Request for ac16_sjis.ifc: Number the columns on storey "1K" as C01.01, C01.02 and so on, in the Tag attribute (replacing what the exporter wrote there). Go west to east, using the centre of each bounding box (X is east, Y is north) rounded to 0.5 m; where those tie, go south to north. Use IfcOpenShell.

First a look at what the model holds.

```python
import ifcopenshell
import ifcopenshell.util.element
import ifcopenshell.util.placement

model = ifcopenshell.open("ac16_sjis.ifc")
print(model.schema)
storey = next(s for s in model.by_type("IfcBuildingStorey") if s.Name == '1\x8aK')
columns = [e for e in ifcopenshell.util.element.get_decomposition(storey) if e.is_a("IfcColumn")]
for e in sorted(columns, key=lambda e: e.id()):
    origin = ifcopenshell.util.placement.get_local_placement(e.ObjectPlacement)[:3, 3]
    print(e.id(), e.Tag, e.Name, origin.round(2) + 0.0, sep=" | ")
```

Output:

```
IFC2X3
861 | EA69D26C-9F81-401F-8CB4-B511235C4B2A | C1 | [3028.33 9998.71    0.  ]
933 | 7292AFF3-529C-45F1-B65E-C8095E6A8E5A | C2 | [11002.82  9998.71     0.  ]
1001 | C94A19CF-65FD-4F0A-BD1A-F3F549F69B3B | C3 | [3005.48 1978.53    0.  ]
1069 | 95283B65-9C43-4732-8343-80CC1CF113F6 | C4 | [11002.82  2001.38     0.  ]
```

```python
import ifcopenshell
import ifcopenshell.geom
import ifcopenshell.util.element
import ifcopenshell.util.shape

model = ifcopenshell.open("ac16_sjis.ifc")
settings = ifcopenshell.geom.settings()
settings.set("use-world-coords", True)


def centre(element):
    shape = ifcopenshell.geom.create_shape(settings, element)
    return ifcopenshell.util.shape.get_bbox_centroid(shape.geometry)


storey = next(s for s in model.by_type("IfcBuildingStorey") if s.Name == '1\x8aK')
columns = [e for e in ifcopenshell.util.element.get_decomposition(storey) if e.is_a("IfcColumn")]

# Insertion points can sit at a corner or the storey origin, so sort by the geometry (in metres).
centres = {e: centre(e) for e in columns}
columns.sort(key=lambda e: (round(centres[e][0] / 0.5), centres[e][1]))

for i, e in enumerate(columns, start=1):
    number = f"C01.{i:02d}"
    e.Tag = number
    print(e.id(), number)

model.write("ac16_sjis_rev.ifc")
```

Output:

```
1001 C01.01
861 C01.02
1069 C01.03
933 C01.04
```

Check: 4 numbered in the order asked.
